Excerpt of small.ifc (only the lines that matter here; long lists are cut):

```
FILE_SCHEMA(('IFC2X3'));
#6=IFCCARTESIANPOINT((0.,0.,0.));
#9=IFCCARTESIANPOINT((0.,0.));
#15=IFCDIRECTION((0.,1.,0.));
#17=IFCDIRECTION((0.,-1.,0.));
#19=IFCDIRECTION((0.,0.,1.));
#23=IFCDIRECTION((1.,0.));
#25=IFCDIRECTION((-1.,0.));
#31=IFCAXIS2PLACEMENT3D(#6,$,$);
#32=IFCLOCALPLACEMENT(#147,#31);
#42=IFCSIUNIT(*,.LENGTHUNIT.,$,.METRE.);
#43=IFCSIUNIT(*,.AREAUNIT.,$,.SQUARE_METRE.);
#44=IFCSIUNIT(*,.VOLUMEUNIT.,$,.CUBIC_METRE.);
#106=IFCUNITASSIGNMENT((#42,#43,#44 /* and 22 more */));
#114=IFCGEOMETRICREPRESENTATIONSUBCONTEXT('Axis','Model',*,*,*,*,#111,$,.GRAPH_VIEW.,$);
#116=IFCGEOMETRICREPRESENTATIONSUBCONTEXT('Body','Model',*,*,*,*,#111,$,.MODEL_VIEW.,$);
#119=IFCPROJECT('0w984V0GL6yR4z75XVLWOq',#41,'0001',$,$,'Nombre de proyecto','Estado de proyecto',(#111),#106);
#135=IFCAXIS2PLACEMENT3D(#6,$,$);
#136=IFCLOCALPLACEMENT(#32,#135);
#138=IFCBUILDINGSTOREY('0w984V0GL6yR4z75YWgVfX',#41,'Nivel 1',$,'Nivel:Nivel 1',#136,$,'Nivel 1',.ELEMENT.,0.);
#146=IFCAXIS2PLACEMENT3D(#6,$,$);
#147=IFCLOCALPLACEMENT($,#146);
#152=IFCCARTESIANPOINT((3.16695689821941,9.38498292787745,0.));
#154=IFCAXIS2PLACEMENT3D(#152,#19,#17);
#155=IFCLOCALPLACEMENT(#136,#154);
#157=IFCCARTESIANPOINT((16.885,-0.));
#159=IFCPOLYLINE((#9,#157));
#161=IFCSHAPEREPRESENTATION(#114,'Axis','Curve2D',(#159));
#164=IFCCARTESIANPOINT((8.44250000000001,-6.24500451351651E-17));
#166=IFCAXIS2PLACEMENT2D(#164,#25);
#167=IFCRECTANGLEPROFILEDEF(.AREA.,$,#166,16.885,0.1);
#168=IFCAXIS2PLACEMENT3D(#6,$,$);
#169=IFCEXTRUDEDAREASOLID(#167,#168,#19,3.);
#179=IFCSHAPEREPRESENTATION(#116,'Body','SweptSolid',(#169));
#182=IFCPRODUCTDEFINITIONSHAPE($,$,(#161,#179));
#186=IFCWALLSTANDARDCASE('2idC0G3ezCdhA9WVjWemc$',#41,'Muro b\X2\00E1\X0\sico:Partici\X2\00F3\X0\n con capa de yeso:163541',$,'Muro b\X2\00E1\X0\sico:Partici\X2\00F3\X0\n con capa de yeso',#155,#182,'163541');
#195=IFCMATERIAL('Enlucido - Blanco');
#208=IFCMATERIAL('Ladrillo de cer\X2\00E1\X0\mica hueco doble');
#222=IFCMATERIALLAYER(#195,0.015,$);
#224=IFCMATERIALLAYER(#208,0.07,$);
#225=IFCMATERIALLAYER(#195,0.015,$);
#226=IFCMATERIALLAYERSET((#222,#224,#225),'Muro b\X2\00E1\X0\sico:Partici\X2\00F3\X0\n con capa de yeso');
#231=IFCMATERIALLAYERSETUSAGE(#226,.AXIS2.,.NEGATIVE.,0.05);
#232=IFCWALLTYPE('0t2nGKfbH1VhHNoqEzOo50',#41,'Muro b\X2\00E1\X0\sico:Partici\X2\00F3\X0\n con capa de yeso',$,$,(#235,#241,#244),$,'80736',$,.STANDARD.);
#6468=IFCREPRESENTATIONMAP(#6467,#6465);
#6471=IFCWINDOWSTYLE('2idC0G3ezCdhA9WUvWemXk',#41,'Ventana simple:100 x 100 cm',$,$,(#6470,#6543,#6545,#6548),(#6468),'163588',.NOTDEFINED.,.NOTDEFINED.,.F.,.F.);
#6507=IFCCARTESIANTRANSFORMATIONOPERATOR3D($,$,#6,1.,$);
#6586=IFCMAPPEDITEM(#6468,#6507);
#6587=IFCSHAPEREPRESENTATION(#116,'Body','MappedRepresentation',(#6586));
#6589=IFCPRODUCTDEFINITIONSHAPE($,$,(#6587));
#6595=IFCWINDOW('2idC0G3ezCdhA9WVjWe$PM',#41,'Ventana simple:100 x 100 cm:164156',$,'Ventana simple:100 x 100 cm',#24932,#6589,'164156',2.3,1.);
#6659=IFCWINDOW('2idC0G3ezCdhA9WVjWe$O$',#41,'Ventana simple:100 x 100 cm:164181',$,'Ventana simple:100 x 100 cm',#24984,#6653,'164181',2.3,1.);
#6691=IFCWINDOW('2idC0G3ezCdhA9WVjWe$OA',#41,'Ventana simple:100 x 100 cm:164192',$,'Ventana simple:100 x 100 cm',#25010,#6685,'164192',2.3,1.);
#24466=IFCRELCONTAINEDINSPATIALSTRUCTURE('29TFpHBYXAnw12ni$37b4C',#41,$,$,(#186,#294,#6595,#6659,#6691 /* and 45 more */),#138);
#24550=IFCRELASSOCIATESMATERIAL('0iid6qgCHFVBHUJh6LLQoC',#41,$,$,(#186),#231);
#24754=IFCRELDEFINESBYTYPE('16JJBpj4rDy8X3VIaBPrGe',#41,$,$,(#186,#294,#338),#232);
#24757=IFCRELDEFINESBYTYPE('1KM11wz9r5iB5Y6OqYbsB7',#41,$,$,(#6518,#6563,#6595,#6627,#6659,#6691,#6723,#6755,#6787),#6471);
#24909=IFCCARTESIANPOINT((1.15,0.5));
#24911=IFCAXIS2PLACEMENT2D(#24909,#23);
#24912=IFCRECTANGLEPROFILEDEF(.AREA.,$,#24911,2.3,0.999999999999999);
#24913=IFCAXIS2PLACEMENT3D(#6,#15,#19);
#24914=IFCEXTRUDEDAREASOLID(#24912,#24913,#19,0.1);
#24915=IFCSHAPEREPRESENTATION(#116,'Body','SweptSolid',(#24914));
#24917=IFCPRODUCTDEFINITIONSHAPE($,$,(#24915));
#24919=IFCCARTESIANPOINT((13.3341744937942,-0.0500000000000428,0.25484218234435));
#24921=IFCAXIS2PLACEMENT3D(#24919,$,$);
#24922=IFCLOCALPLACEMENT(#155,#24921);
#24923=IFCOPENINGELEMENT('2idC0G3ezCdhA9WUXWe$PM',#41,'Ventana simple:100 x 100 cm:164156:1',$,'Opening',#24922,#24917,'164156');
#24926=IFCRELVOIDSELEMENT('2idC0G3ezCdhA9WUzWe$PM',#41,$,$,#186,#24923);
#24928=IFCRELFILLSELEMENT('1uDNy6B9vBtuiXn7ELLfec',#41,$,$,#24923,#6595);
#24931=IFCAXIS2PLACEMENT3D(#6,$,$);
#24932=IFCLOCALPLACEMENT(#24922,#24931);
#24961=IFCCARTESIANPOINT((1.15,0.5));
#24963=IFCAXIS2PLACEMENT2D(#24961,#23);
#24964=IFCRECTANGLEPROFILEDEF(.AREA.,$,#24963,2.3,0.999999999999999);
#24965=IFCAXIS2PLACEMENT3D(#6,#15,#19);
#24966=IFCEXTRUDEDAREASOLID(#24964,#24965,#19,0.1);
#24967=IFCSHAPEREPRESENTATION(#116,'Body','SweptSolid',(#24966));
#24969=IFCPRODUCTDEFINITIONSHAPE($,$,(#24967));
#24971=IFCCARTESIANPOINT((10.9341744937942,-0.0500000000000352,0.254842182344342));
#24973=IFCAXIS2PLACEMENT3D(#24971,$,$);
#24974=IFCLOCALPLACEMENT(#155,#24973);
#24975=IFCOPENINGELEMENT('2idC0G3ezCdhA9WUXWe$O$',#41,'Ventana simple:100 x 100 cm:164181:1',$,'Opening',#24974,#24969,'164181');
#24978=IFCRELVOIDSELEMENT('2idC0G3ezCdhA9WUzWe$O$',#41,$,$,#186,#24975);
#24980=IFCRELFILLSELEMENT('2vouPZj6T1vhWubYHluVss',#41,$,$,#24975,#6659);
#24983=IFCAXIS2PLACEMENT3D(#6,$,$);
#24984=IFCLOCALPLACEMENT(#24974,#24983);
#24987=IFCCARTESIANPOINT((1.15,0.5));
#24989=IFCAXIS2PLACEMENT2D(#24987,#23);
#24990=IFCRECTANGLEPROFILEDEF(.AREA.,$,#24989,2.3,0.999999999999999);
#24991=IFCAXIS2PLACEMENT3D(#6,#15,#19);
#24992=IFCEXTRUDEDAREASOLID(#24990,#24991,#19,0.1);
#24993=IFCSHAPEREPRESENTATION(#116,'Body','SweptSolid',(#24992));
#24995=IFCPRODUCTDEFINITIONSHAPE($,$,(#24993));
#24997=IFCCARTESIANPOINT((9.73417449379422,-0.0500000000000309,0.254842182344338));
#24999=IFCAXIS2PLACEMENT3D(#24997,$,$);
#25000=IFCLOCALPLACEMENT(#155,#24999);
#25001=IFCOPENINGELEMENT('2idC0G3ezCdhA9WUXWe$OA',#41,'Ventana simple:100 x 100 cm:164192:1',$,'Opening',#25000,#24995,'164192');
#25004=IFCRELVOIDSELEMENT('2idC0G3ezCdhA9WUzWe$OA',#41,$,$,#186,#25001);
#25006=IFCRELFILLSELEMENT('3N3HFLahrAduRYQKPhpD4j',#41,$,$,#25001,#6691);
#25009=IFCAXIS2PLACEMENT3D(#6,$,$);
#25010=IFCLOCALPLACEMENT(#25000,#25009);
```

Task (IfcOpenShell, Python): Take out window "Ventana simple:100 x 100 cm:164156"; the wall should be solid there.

```python
import ifcopenshell
import ifcopenshell.api.feature
import ifcopenshell.api.root
import ifcopenshell.geom
import ifcopenshell.util.shape

model = ifcopenshell.open("small.ifc")
settings = ifcopenshell.geom.settings()


def volume(element):
    """Net volume in cubic metres, openings subtracted."""
    shape = ifcopenshell.geom.create_shape(settings, element)
    return ifcopenshell.util.shape.get_volume(shape.geometry)


window = model.by_guid("2idC0G3ezCdhA9WVjWe$PM")
opening = window.FillsVoids[0].RelatingOpeningElement
wall = opening.VoidsElements[0].RelatingBuildingElement
before = volume(wall)

ifcopenshell.api.root.remove_product(model, product=window)
ifcopenshell.api.feature.remove_feature(model, feature=opening)

after = volume(wall)

print(f"wall volume {before:.3f} -> {after:.3f} m3")

model.write("small_updated.ifc")
```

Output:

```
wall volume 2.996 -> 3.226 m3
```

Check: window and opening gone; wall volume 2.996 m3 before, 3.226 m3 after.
